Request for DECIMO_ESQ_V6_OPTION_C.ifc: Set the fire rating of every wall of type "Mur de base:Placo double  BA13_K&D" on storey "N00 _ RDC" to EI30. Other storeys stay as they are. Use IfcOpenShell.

First a look at what the model holds.

```python
import ifcopenshell
import ifcopenshell.util.element

model = ifcopenshell.open("DECIMO_ESQ_V6_OPTION_C.ifc")
print(model.schema)
storey = next(s for s in model.by_type("IfcBuildingStorey") if s.Name == "N00 _ RDC")
walls = [e for e in ifcopenshell.util.element.get_decomposition(storey) if e.is_a("IfcWall")]
seen = {}
for e in walls:
    element_type = ifcopenshell.util.element.get_type(e)
    key = (element_type.Name if element_type != e and element_type else None, ifcopenshell.util.element.get_pset(e, "Pset_WallCommon", "FireRating"))
    seen[key] = seen.get(key, 0) + 1
for (name, value), count in sorted(seen.items(), key=str):
    print(count, "x", name, "|", value)
```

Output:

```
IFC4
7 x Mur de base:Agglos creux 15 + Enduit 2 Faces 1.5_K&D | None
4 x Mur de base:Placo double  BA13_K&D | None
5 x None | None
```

```python
import ifcopenshell
import ifcopenshell.api.pset
import ifcopenshell.util.element

model = ifcopenshell.open("DECIMO_ESQ_V6_OPTION_C.ifc")

storey = next(s for s in model.by_type("IfcBuildingStorey") if s.Name == "N00 _ RDC")
walls = [e for e in ifcopenshell.util.element.get_decomposition(storey) if e.is_a("IfcWall")]

count = 0
for e in walls:
    element_type = ifcopenshell.util.element.get_type(e)
    if element_type in (None, e) or element_type.Name != "Mur de base:Placo double  BA13_K&D":
        continue
    # add_pset returns the element's existing set when there is one.
    pset = ifcopenshell.api.pset.add_pset(model, product=e, name="Pset_WallCommon")
    ifcopenshell.api.pset.edit_pset(model, pset=pset, properties={"FireRating": "EI30"})
    count += 1

print(count, "walls updated")

model.write("DECIMO_ESQ_V6_OPTION_C_edited.ifc")
```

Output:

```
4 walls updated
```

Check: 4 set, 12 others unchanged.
